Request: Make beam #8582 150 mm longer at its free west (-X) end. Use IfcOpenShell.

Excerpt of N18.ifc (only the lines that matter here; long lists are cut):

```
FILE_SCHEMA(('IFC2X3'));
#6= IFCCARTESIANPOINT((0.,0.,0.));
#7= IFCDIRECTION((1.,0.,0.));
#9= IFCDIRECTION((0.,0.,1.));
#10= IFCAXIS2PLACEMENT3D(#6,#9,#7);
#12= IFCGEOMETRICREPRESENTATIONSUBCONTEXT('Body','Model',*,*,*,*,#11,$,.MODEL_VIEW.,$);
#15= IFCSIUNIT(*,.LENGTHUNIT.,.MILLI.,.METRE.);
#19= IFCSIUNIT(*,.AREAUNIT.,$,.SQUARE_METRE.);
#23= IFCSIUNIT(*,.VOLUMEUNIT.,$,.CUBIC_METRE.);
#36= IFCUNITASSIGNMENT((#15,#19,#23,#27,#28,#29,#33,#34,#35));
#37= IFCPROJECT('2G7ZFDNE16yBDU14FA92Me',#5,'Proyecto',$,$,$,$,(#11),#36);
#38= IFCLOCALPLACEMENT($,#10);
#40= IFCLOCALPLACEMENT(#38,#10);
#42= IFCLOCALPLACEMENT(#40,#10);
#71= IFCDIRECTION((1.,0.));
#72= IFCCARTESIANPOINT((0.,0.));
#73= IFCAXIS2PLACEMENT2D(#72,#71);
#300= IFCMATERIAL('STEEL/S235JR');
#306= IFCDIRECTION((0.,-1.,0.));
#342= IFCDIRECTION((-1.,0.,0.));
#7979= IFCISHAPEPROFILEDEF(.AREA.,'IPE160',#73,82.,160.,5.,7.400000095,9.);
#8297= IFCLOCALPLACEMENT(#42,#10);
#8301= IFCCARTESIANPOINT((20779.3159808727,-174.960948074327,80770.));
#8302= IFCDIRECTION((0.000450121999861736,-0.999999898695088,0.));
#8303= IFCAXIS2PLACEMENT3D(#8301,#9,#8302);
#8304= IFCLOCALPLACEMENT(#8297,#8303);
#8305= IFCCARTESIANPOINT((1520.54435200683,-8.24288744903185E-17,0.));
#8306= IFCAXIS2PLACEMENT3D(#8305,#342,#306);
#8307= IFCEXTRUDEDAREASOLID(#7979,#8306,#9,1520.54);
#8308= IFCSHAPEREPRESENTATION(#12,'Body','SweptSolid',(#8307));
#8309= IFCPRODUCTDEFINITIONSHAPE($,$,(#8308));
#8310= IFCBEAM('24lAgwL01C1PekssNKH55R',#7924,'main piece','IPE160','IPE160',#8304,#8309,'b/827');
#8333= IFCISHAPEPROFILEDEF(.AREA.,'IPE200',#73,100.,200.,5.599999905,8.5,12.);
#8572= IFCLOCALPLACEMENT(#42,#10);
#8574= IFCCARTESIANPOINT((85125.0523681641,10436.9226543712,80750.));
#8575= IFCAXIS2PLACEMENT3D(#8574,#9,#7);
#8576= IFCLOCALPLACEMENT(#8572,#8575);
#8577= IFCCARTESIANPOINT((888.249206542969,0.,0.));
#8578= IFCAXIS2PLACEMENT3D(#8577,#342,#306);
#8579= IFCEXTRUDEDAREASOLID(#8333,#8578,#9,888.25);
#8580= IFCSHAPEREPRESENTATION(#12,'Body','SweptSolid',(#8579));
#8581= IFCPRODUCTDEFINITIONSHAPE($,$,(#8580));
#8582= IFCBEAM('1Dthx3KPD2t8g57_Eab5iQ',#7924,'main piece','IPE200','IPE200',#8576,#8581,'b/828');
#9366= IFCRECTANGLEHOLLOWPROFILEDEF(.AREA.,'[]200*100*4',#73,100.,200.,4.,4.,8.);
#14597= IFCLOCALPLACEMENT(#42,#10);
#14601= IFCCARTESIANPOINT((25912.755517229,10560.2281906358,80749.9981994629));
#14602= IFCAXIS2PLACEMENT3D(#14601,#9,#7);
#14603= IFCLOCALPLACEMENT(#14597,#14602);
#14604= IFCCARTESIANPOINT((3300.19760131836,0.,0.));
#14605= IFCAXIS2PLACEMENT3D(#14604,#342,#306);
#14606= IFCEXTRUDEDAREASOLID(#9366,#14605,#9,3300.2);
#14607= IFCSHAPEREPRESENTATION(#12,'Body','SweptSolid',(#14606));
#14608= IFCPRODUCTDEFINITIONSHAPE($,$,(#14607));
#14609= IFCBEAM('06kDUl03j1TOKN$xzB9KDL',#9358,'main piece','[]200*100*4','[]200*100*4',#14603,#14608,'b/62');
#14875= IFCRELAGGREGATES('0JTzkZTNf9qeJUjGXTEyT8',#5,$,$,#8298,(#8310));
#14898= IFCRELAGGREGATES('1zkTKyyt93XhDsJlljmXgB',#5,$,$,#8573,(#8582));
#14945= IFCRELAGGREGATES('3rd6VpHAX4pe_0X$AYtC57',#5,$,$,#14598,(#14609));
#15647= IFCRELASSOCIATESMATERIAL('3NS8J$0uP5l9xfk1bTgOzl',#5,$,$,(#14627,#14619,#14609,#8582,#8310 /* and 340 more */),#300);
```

```python
import ifcopenshell
import ifcopenshell.util.representation
import ifcopenshell.util.unit

model = ifcopenshell.open("N18.ifc")
unit_scale = ifcopenshell.util.unit.calculate_unit_scale(model)

member = model.by_guid("1Dthx3KPD2t8g57_Eab5iQ")
change = 0.15 / unit_scale

# The extrusion runs towards the end named, so only its depth changes.
body = ifcopenshell.util.representation.get_representation(member, "Model", "Body")
solid = body.Items[0]
old_length = solid.Depth
solid.Depth += change

print(f"length {old_length:g} -> {solid.Depth:g}")

model.write("N18_v2.ifc")
```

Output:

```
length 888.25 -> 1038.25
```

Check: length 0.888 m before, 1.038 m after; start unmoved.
